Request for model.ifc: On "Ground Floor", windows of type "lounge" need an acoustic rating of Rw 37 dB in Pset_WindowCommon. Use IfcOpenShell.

First a look at what the model holds.

```python
import ifcopenshell
import ifcopenshell.util.element

model = ifcopenshell.open("model.ifc")
print(model.schema)
storey = next(s for s in model.by_type("IfcBuildingStorey") if s.Name == "Ground Floor")
windows = [e for e in ifcopenshell.util.element.get_decomposition(storey) if e.is_a("IfcWindow")]
seen = {}
for e in windows:
    element_type = ifcopenshell.util.element.get_type(e)
    key = (element_type.Name if element_type != e and element_type else None, ifcopenshell.util.element.get_pset(e, "Pset_WindowCommon", "AcousticRating"))
    seen[key] = seen.get(key, 0) + 1
for (name, value), count in sorted(seen.items(), key=str):
    print(count, "x", name, "|", value)
```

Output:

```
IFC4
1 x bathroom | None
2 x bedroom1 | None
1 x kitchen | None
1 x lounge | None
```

```python
import ifcopenshell
import ifcopenshell.api.pset
import ifcopenshell.util.element

model = ifcopenshell.open("model.ifc")

storey = next(s for s in model.by_type("IfcBuildingStorey") if s.Name == "Ground Floor")
windows = [e for e in ifcopenshell.util.element.get_decomposition(storey) if e.is_a("IfcWindow")]

count = 0
for e in windows:
    element_type = ifcopenshell.util.element.get_type(e)
    if element_type in (None, e) or element_type.Name != "lounge":
        continue
    # add_pset returns the element's existing set when there is one.
    pset = ifcopenshell.api.pset.add_pset(model, product=e, name="Pset_WindowCommon")
    ifcopenshell.api.pset.edit_pset(model, pset=pset, properties={"AcousticRating": "Rw 37 dB"})
    count += 1

print(count, "windows updated")

model.write("model_edited.ifc")
```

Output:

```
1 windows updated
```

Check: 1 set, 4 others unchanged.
